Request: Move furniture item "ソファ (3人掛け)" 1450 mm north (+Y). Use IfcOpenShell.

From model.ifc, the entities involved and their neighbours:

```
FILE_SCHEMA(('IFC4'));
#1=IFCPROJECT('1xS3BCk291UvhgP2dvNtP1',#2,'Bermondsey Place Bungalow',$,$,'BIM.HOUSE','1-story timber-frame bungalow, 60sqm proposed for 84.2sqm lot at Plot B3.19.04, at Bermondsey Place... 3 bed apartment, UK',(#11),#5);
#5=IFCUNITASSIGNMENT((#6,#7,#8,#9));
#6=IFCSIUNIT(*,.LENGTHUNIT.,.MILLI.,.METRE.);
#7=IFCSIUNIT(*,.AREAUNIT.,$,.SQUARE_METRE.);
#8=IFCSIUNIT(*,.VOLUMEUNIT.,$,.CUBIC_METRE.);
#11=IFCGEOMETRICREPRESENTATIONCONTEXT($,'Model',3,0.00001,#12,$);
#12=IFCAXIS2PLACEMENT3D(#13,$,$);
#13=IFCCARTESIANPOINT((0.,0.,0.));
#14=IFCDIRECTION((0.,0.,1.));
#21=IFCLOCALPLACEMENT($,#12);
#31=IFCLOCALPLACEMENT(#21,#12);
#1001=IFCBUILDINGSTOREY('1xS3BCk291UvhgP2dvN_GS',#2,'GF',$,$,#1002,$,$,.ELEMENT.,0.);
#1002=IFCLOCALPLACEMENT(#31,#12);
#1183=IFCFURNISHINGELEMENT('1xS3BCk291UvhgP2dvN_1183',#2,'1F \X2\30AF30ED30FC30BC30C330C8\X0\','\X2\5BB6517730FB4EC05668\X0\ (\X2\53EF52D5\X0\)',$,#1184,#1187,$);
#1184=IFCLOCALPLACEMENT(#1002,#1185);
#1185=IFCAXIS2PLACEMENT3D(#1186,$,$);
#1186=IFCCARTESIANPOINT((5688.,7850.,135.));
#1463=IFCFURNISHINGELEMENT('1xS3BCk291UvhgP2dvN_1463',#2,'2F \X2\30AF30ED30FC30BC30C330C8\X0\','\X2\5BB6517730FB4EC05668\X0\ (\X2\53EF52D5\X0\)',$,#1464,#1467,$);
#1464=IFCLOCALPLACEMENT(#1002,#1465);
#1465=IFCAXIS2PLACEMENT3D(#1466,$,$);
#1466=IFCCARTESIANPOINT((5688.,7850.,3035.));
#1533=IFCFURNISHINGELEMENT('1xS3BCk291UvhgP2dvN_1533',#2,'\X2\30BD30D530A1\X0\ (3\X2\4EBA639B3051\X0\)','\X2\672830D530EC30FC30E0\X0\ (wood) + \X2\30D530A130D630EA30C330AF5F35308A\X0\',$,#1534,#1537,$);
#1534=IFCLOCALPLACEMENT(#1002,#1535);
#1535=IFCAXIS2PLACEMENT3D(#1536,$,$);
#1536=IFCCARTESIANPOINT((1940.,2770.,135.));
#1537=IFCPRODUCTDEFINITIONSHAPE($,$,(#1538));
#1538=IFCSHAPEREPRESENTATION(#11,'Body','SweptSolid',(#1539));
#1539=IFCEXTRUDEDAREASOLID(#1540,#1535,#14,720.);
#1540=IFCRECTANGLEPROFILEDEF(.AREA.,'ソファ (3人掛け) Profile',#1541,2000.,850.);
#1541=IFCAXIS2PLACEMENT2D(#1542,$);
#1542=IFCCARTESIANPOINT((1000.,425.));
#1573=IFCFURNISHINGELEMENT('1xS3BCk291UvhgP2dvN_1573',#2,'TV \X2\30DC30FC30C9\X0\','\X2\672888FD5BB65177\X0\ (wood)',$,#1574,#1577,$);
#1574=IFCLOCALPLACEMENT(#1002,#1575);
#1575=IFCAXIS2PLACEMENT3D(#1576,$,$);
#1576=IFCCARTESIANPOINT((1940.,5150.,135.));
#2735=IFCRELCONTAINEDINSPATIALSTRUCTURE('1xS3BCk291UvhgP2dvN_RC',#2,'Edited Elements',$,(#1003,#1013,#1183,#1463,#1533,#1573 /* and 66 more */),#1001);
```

```python
import ifcopenshell
import ifcopenshell.api.geometry
import ifcopenshell.util.placement

model = ifcopenshell.open("model.ifc")

item = model.by_guid("1xS3BCk291UvhgP2dvN_1533")
matrix = ifcopenshell.util.placement.get_local_placement(item.ObjectPlacement)
matrix[1, 3] += 1450.0
ifcopenshell.api.geometry.edit_object_placement(model, product=item, matrix=matrix, is_si=False)

print(ifcopenshell.util.placement.get_local_placement(item.ObjectPlacement).round(3) + 0.0)

model.write("model_rev.ifc")
```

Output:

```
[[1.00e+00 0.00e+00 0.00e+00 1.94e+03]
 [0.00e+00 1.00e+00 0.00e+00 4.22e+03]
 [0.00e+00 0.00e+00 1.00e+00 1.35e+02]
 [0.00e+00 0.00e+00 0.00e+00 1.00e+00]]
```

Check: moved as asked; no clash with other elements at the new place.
